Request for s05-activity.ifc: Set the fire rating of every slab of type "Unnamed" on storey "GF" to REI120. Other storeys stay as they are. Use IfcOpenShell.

First a look at what the model holds.

```python
import ifcopenshell
import ifcopenshell.util.element

model = ifcopenshell.open("s05-activity.ifc")
print(model.schema)
storey = next(s for s in model.by_type("IfcBuildingStorey") if s.Name == "GF")
slabs = [e for e in ifcopenshell.util.element.get_decomposition(storey) if e.is_a("IfcSlab")]
seen = {}
for e in slabs:
    element_type = ifcopenshell.util.element.get_type(e)
    key = (element_type.Name if element_type != e and element_type else None, ifcopenshell.util.element.get_pset(e, "Pset_SlabCommon", "FireRating"))
    seen[key] = seen.get(key, 0) + 1
for (name, value), count in sorted(seen.items(), key=str):
    print(count, "x", name, "|", value)
```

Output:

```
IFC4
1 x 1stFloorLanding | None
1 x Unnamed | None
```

```python
import ifcopenshell
import ifcopenshell.api.pset
import ifcopenshell.util.element

model = ifcopenshell.open("s05-activity.ifc")

storey = next(s for s in model.by_type("IfcBuildingStorey") if s.Name == "GF")
slabs = [e for e in ifcopenshell.util.element.get_decomposition(storey) if e.is_a("IfcSlab")]

count = 0
for e in slabs:
    element_type = ifcopenshell.util.element.get_type(e)
    if element_type in (None, e) or element_type.Name != "Unnamed":
        continue
    # add_pset returns the element's existing set when there is one.
    pset = ifcopenshell.api.pset.add_pset(model, product=e, name="Pset_SlabCommon")
    ifcopenshell.api.pset.edit_pset(model, pset=pset, properties={"FireRating": "REI120"})
    count += 1

print(count, "slabs updated")

model.write("s05-activity_v2.ifc")
```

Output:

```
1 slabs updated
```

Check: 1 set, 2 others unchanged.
